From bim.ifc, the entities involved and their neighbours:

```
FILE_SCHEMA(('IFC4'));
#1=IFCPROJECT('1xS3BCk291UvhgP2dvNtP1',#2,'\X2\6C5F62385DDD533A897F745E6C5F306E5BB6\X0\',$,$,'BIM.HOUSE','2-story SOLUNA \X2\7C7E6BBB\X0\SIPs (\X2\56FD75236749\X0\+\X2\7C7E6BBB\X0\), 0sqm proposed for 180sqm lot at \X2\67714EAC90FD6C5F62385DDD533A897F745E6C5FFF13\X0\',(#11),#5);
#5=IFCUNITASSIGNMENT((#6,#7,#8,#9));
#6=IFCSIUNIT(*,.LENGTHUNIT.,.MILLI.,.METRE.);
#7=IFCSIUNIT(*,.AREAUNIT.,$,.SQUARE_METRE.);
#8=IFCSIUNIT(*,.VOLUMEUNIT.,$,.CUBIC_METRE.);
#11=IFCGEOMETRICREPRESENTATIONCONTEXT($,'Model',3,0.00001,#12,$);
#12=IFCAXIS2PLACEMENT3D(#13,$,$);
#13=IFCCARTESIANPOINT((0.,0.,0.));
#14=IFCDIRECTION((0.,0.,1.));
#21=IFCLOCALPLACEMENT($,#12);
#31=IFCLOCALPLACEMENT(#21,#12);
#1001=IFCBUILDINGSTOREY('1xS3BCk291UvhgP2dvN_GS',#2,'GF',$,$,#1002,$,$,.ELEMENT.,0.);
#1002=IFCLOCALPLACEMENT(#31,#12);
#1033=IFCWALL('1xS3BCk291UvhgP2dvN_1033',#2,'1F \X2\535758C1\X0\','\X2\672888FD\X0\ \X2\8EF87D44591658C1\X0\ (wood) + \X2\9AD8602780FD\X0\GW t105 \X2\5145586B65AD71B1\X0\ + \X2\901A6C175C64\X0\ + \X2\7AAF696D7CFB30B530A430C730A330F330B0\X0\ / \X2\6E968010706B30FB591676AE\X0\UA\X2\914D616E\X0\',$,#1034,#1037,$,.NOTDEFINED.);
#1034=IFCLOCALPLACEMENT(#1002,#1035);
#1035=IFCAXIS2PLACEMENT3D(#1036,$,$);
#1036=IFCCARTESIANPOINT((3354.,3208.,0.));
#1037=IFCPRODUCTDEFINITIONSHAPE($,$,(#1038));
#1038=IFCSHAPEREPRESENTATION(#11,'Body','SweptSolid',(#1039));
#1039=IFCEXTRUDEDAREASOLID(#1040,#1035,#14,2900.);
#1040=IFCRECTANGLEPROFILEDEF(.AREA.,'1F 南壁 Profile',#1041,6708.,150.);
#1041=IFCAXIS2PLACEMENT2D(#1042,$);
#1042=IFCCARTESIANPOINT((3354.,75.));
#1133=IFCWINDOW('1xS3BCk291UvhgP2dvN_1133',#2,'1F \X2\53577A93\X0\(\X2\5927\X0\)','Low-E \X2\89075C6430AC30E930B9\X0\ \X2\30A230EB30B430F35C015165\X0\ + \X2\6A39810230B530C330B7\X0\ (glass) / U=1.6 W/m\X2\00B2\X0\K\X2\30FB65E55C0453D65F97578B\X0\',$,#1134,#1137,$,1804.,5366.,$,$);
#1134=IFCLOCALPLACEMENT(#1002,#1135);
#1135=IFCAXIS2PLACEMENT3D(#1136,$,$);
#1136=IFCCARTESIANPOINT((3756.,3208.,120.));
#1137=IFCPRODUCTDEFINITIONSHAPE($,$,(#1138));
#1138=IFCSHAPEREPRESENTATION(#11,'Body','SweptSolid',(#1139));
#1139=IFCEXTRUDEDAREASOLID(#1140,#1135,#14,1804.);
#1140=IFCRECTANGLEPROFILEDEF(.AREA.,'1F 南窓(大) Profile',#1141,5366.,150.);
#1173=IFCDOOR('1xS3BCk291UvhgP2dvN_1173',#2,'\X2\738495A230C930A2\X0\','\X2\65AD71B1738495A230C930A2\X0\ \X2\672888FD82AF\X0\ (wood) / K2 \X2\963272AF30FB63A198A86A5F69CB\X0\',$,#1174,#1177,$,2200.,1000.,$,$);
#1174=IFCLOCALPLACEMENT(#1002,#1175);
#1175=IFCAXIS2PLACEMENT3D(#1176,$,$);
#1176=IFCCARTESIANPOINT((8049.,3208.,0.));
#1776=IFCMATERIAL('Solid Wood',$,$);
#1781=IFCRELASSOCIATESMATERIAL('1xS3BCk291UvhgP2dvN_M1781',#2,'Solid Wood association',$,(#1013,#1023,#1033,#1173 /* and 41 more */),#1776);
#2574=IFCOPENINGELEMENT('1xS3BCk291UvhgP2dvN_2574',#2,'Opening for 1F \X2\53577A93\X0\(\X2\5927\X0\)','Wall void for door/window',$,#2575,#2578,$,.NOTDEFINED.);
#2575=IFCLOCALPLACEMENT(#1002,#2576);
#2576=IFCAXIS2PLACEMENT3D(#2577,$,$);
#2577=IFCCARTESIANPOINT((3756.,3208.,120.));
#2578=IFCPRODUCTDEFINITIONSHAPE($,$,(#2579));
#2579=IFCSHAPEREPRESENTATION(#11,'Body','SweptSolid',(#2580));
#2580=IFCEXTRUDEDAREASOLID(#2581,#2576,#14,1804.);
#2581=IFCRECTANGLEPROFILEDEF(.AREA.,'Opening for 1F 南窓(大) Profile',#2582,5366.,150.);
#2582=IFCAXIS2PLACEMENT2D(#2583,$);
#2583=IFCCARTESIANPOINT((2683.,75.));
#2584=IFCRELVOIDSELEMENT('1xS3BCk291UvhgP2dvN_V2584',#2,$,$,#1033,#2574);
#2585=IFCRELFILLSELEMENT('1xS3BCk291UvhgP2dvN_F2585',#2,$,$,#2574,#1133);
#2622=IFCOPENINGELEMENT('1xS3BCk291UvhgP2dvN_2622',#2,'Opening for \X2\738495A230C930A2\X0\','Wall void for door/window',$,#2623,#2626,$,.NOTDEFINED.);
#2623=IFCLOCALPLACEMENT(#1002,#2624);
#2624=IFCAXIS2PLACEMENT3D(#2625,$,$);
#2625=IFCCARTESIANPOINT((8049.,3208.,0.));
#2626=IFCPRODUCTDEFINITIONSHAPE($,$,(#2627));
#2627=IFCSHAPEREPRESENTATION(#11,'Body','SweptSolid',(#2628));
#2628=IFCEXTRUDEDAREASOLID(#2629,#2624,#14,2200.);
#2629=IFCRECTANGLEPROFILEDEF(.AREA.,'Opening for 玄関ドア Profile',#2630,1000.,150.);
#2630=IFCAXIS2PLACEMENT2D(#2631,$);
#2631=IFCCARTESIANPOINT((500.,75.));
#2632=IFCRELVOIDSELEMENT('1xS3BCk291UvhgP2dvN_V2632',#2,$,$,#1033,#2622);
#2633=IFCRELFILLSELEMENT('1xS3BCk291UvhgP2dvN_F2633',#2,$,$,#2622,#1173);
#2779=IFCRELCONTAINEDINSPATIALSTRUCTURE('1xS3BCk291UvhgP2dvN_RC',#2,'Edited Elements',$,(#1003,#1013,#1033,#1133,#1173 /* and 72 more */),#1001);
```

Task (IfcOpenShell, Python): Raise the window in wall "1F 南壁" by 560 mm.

```python
import numpy as np
import ifcopenshell
import ifcopenshell.api.geometry
import ifcopenshell.util.placement
import ifcopenshell.util.unit

model = ifcopenshell.open("bim.ifc")
unit_scale = ifcopenshell.util.unit.calculate_unit_scale(model)

window = model.by_guid("1xS3BCk291UvhgP2dvN_1133")
opening = window.FillsVoids[0].RelatingOpeningElement
dz = 560.0

shift = np.array([0.0, 0.0, dz])
# The window is not placed relative to its opening, so move both.
for product in (opening, window):
    matrix = ifcopenshell.util.placement.get_local_placement(product.ObjectPlacement)
    matrix[:3, 3] += shift
    ifcopenshell.api.geometry.edit_object_placement(model, product=product, matrix=matrix, is_si=False)

print(f"moved by {dz * unit_scale:+.3f} m")

model.write("bim-out.ifc")
```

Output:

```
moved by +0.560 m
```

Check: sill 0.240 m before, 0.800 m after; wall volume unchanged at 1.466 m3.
